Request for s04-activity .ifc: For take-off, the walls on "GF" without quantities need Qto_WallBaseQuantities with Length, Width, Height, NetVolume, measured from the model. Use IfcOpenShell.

First a look at what the model holds.

```python
import ifcopenshell
import ifcopenshell.util.element
import ifcopenshell.util.unit

model = ifcopenshell.open("s04-activity .ifc")
print(model.schema)
for unit_type in ("LENGTHUNIT", "AREAUNIT", "VOLUMEUNIT"):
    print(unit_type, ifcopenshell.util.unit.calculate_unit_scale(model, unit_type))
storey = next(s for s in model.by_type("IfcBuildingStorey") if s.Name == "GF")
walls = [e for e in ifcopenshell.util.element.get_decomposition(storey) if e.is_a("IfcWall")]
for e in sorted(walls, key=lambda e: e.id()):
    print(e.id(), e.is_a(), e.Name, list(ifcopenshell.util.element.get_psets(e, qtos_only=True)), sep=" | ")
```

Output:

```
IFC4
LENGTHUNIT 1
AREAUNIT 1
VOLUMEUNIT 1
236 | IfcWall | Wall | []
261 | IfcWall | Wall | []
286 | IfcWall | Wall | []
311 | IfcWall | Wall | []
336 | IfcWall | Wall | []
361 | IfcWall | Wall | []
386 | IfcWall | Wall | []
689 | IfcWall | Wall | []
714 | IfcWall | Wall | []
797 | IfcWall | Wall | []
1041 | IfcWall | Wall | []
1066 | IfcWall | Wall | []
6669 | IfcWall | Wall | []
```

```python
import ifcopenshell
import ifcopenshell.api.pset
import ifcopenshell.geom
import ifcopenshell.util.element
import ifcopenshell.util.shape
import ifcopenshell.util.unit

model = ifcopenshell.open("s04-activity .ifc")
unit_scale = ifcopenshell.util.unit.calculate_unit_scale(model)
volume_scale = ifcopenshell.util.unit.calculate_unit_scale(model, "VOLUMEUNIT")
settings = ifcopenshell.geom.settings()

storey = next(s for s in model.by_type("IfcBuildingStorey") if s.Name == "GF")
walls = [e for e in ifcopenshell.util.element.get_decomposition(storey) if e.is_a("IfcWall")]

for e in sorted(walls, key=lambda e: e.id()):
    if ifcopenshell.util.element.get_psets(e, qtos_only=True, should_inherit=False):
        continue
    # Geometry comes back in metres, in the element's own axes.
    shape = ifcopenshell.geom.create_shape(settings, e)
    values = {
        "Length": ifcopenshell.util.shape.get_x(shape.geometry) / unit_scale,
        "Width": ifcopenshell.util.shape.get_y(shape.geometry) / unit_scale,
        "Height": ifcopenshell.util.shape.get_z(shape.geometry) / unit_scale,
        "NetVolume": ifcopenshell.util.shape.get_volume(shape.geometry) / volume_scale,
    }
    qto = ifcopenshell.api.pset.add_qto(model, product=e, name="Qto_WallBaseQuantities")
    ifcopenshell.api.pset.edit_qto(model, qto=qto, properties=values)
    print(e.id(), {k: round(v, 3) for k, v in values.items()})

model.write("s04-activity _updated.ifc")
```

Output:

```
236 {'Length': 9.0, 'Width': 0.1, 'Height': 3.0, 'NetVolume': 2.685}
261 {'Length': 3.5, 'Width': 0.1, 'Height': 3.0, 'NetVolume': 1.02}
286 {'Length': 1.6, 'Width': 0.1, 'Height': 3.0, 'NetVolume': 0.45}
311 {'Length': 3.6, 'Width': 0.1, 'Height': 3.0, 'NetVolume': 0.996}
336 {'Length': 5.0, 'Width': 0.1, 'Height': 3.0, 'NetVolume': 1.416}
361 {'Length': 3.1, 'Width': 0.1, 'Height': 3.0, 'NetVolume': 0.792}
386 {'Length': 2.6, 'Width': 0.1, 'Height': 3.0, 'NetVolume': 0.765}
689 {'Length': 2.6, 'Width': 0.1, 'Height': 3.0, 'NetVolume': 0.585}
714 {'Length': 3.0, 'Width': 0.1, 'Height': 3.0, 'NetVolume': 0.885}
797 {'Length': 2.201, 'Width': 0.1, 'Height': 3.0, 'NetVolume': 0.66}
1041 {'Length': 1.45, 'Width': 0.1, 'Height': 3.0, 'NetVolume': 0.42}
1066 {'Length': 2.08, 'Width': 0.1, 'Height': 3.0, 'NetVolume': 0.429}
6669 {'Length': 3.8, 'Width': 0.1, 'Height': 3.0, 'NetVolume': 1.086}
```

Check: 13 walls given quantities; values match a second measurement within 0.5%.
